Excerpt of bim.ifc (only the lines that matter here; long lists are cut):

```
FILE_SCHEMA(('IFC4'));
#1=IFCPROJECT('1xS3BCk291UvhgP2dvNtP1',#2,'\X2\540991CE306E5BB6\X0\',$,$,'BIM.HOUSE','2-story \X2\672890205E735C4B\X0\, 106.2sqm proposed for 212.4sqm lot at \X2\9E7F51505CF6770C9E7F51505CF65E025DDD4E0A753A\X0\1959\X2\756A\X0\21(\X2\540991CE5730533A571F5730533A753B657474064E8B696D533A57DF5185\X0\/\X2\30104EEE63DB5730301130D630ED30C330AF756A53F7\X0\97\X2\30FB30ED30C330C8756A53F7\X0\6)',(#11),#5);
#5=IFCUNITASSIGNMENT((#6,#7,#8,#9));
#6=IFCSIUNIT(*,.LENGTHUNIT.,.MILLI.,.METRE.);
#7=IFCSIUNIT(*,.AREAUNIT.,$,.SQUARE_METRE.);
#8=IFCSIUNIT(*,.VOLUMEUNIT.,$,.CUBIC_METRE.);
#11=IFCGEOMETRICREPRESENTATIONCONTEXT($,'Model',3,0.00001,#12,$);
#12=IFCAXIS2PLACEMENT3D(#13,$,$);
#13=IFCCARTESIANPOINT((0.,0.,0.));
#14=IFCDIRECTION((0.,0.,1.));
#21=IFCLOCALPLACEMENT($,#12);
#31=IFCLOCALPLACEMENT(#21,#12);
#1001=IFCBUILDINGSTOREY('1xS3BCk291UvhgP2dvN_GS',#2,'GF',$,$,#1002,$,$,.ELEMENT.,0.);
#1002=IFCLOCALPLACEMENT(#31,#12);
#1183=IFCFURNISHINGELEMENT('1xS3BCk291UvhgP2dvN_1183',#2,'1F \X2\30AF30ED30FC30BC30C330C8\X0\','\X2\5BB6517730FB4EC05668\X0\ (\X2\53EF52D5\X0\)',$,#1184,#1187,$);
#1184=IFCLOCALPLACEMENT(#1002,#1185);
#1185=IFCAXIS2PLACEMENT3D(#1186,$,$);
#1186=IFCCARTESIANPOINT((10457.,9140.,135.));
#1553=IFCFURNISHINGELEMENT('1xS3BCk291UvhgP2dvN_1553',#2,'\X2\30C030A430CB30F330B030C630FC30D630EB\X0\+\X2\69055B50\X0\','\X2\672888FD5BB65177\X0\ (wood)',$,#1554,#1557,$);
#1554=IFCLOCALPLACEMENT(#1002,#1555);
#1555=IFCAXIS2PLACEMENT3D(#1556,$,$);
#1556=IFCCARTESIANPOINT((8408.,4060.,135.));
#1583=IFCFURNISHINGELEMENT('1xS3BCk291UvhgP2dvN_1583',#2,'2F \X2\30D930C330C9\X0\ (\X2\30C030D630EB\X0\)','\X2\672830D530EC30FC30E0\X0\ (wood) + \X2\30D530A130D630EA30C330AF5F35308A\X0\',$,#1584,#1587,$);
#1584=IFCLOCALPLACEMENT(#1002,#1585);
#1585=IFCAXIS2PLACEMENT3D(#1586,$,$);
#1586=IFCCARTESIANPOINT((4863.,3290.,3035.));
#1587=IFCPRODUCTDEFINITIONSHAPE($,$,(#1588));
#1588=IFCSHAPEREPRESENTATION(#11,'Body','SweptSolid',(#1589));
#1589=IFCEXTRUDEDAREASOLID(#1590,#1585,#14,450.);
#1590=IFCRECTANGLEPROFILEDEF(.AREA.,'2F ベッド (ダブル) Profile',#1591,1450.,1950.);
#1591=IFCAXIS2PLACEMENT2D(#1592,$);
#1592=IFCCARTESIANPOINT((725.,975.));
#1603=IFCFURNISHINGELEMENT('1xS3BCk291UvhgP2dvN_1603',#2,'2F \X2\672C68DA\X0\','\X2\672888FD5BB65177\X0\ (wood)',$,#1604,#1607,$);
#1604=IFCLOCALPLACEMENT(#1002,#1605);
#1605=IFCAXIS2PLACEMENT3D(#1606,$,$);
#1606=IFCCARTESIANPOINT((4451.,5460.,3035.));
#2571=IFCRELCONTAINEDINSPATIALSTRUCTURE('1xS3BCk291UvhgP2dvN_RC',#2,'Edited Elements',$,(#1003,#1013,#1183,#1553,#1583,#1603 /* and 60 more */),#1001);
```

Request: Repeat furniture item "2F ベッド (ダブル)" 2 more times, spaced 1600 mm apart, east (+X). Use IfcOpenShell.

```python
import numpy as np
import ifcopenshell
import ifcopenshell.api.geometry
import ifcopenshell.api.root
import ifcopenshell.util.element
import ifcopenshell.util.placement

model = ifcopenshell.open("bim.ifc")


def reuse_history(source, copy):
    """copy_class also copies each property set's owner history, people and application; keep the originals."""
    for rel in copy.IsDefinedBy:
        if rel.is_a("IfcRelDefinesByProperties") and (history := rel.RelatingPropertyDefinition.OwnerHistory):
            rel.RelatingPropertyDefinition.OwnerHistory = source.OwnerHistory
            ifcopenshell.util.element.remove_deep2(model, history)


source = model.by_guid("1xS3BCk291UvhgP2dvN_1583")
base = ifcopenshell.util.placement.get_local_placement(source.ObjectPlacement)
step = np.array([1.0, 0.0, 0.0]) * 1600.0

for i in range(1, 3):
    copy = ifcopenshell.api.root.copy_class(model, product=source)
    copy.Representation = ifcopenshell.util.element.copy_deep(
        model, source.Representation, exclude=["IfcGeometricRepresentationContext", "IfcRepresentationMap"]
    )
    reuse_history(source, copy)
    matrix = base.copy()
    matrix[:3, 3] += i * step
    print("added at", matrix[:3, 3].round(3) + 0.0)
    ifcopenshell.api.geometry.edit_object_placement(model, product=copy, matrix=matrix, is_si=False)

model.write("bim-out.ifc")
```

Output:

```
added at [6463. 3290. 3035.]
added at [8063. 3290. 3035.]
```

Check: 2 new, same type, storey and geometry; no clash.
